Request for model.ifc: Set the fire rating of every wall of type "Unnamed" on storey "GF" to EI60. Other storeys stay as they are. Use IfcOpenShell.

First a look at what the model holds.

```python
import ifcopenshell
import ifcopenshell.util.element

model = ifcopenshell.open("model.ifc")
print(model.schema)
storey = next(s for s in model.by_type("IfcBuildingStorey") if s.Name == "GF")
walls = [e for e in ifcopenshell.util.element.get_decomposition(storey) if e.is_a("IfcWall")]
seen = {}
for e in walls:
    element_type = ifcopenshell.util.element.get_type(e)
    key = (element_type.Name if element_type != e and element_type else None, ifcopenshell.util.element.get_pset(e, "Pset_WallCommon", "FireRating"))
    seen[key] = seen.get(key, 0) + 1
for (name, value), count in sorted(seen.items(), key=str):
    print(count, "x", name, "|", value)
```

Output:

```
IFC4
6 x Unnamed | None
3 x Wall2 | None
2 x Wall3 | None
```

```python
import ifcopenshell
import ifcopenshell.api.pset
import ifcopenshell.util.element

model = ifcopenshell.open("model.ifc")

storey = next(s for s in model.by_type("IfcBuildingStorey") if s.Name == "GF")
walls = [e for e in ifcopenshell.util.element.get_decomposition(storey) if e.is_a("IfcWall")]

count = 0
for e in walls:
    element_type = ifcopenshell.util.element.get_type(e)
    if element_type in (None, e) or element_type.Name != "Unnamed":
        continue
    # add_pset returns the element's existing set when there is one.
    pset = ifcopenshell.api.pset.add_pset(model, product=e, name="Pset_WallCommon")
    ifcopenshell.api.pset.edit_pset(model, pset=pset, properties={"FireRating": "EI60"})
    count += 1

print(count, "walls updated")

model.write("model-out.ifc")
```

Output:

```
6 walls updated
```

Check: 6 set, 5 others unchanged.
